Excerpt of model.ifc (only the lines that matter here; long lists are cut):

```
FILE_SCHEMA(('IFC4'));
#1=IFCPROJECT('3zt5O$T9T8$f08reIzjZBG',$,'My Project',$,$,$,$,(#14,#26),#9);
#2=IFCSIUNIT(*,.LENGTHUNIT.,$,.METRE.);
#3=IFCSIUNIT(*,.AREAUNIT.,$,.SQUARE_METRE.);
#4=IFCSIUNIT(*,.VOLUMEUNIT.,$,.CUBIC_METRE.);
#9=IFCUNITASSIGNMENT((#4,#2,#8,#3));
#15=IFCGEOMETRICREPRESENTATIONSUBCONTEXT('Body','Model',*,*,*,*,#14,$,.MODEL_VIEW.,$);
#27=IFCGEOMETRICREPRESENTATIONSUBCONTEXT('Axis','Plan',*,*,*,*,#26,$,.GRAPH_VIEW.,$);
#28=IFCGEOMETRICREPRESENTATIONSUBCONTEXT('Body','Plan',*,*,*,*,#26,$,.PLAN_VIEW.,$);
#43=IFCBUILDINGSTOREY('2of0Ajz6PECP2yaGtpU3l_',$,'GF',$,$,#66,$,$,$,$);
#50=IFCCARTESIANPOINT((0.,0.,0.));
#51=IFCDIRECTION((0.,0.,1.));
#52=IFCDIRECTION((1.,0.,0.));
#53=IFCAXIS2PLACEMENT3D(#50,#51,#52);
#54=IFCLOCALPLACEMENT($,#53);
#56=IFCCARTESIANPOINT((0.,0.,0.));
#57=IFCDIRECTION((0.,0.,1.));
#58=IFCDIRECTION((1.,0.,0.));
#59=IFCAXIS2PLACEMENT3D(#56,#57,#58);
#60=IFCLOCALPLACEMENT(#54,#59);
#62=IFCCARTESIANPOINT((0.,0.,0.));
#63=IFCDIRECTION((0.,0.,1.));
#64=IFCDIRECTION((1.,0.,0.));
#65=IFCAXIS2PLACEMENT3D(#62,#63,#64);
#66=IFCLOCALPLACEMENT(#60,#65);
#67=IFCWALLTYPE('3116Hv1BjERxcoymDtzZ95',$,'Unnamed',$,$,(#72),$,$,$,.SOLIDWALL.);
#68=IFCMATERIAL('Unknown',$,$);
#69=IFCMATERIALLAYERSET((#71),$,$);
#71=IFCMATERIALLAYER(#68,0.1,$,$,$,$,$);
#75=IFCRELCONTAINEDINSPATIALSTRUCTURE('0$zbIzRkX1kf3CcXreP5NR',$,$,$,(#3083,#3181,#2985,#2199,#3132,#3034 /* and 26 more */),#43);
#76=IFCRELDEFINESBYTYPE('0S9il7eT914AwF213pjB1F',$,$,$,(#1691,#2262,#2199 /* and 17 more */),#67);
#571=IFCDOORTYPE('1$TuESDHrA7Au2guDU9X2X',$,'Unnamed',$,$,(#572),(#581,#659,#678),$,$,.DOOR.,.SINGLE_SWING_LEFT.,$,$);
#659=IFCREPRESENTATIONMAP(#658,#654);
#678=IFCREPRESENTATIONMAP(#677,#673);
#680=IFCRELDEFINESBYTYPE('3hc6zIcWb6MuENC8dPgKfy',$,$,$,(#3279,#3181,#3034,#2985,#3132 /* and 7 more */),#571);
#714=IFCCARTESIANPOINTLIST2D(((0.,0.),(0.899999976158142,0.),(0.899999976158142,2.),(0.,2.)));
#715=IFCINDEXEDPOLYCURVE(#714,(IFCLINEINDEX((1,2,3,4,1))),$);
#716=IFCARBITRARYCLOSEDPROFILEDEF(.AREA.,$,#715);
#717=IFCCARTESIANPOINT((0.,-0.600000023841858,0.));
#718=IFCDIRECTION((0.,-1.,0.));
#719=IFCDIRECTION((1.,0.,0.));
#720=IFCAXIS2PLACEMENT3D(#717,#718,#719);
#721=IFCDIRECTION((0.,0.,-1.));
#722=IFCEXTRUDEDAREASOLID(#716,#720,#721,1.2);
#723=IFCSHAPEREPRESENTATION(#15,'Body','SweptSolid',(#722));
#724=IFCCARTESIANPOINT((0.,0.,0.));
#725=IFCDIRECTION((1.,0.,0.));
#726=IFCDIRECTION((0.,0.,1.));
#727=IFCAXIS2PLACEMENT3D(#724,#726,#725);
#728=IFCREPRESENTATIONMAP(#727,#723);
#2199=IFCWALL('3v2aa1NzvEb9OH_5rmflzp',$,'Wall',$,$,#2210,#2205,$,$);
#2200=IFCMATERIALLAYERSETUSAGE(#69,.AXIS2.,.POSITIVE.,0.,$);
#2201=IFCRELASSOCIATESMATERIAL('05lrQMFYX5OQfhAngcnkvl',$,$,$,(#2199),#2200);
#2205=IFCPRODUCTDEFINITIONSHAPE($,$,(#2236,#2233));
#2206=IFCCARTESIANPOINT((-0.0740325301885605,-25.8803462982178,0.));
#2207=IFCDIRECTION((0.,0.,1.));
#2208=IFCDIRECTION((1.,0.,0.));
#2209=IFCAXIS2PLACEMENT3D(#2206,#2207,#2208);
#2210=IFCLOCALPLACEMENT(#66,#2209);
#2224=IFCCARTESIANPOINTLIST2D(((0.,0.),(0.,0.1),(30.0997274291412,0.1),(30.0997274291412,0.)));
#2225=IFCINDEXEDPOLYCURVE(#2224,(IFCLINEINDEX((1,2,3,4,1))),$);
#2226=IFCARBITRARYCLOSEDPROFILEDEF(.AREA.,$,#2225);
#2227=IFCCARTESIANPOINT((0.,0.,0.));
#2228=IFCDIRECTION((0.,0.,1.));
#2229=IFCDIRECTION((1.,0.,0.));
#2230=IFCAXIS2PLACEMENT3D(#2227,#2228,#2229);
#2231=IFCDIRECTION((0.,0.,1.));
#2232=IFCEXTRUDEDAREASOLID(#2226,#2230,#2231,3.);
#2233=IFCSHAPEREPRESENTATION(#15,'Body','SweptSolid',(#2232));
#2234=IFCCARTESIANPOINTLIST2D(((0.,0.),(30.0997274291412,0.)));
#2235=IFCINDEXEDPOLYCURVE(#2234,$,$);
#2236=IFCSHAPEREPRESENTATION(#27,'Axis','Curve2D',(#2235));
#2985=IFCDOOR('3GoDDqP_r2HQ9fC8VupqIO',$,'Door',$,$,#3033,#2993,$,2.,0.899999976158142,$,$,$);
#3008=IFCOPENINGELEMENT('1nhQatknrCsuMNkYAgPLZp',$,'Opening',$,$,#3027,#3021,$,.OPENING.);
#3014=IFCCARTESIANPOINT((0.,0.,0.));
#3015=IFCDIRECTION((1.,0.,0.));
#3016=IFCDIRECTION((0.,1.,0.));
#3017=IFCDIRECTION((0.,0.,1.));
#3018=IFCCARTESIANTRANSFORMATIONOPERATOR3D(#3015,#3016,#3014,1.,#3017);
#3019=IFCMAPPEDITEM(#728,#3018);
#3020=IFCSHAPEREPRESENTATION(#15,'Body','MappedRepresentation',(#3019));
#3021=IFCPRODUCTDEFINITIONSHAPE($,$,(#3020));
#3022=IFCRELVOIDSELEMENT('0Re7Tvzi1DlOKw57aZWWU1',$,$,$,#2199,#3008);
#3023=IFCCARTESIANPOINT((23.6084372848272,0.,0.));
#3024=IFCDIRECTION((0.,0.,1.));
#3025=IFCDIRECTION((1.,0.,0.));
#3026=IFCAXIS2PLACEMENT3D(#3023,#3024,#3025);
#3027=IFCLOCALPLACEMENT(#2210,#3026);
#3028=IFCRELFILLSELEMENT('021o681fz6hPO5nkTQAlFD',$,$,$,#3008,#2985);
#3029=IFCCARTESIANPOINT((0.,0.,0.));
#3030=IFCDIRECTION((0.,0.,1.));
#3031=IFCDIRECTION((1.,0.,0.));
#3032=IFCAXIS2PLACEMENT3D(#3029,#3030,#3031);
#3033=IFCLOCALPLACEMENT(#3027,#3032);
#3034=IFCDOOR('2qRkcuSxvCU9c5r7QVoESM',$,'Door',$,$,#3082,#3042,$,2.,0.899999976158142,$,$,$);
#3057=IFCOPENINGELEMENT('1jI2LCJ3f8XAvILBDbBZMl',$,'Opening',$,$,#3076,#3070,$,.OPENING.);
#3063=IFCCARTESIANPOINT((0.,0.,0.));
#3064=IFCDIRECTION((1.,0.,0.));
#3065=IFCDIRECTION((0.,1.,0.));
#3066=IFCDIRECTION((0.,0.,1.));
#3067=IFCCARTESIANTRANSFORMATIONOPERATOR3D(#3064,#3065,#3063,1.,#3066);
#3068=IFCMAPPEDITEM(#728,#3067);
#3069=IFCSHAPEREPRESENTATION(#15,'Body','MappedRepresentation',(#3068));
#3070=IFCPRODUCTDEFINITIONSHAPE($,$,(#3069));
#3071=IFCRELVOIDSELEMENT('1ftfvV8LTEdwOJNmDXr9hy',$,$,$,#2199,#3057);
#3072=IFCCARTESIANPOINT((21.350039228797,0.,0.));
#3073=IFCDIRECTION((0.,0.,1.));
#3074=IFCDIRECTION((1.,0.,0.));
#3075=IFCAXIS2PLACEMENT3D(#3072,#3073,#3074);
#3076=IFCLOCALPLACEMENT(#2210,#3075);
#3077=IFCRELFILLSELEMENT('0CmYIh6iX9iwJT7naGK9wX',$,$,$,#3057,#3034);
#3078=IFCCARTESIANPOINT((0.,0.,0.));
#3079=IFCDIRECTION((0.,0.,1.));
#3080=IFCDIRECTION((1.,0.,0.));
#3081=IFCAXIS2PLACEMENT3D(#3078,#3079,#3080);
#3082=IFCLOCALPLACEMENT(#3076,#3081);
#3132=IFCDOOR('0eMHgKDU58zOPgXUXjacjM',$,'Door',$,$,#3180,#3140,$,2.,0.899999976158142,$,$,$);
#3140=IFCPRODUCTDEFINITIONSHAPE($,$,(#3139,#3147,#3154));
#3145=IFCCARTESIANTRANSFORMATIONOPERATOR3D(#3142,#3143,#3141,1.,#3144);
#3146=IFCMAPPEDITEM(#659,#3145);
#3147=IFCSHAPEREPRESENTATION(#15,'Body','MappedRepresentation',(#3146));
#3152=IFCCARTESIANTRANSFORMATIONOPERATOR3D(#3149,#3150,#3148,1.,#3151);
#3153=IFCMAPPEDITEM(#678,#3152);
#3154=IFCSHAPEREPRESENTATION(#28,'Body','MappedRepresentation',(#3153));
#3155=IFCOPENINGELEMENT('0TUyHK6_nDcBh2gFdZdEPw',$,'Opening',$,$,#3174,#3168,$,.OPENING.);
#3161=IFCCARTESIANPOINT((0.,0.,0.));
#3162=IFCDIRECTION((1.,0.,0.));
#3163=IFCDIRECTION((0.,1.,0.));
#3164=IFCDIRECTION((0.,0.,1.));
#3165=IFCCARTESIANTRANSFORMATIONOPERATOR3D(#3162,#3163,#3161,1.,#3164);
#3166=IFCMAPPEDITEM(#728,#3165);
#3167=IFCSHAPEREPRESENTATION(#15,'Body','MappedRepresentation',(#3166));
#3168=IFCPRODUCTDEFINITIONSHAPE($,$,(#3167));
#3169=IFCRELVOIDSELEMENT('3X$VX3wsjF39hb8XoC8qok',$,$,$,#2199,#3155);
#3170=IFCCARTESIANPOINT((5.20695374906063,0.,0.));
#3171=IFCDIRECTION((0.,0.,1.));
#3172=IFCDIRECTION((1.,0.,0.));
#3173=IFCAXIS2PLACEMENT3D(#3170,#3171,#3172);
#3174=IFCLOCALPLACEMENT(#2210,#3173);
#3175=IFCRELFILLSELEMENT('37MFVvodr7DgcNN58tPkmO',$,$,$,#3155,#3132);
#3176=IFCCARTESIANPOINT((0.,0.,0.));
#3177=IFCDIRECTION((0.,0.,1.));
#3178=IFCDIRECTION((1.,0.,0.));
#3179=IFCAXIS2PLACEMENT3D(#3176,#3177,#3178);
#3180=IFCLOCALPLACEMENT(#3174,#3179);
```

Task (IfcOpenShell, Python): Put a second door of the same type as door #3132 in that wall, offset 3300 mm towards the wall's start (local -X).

```python
import ifcopenshell
import ifcopenshell.api.feature
import ifcopenshell.api.geometry
import ifcopenshell.api.root
import ifcopenshell.geom
import ifcopenshell.util.element
import ifcopenshell.util.placement
import ifcopenshell.util.shape
import ifcopenshell.util.unit

model = ifcopenshell.open("model.ifc")
unit_scale = ifcopenshell.util.unit.calculate_unit_scale(model)
settings = ifcopenshell.geom.settings()


def volume(element):
    """Net volume in cubic metres, openings subtracted."""
    shape = ifcopenshell.geom.create_shape(settings, element)
    return ifcopenshell.util.shape.get_volume(shape.geometry)


door = model.by_guid("0eMHgKDU58zOPgXUXjacjM")
opening = door.FillsVoids[0].RelatingOpeningElement
wall = opening.VoidsElements[0].RelatingBuildingElement
before = volume(wall)
shift = ifcopenshell.util.placement.get_local_placement(wall.ObjectPlacement)[:3, 0] * -3.3 / unit_scale

# copy_class copies the void relationship, type, container and properties, but no geometry.
new_opening = ifcopenshell.api.root.copy_class(model, product=opening)
new_opening.Representation = ifcopenshell.util.element.copy_deep(
    model, opening.Representation, exclude=["IfcGeometricRepresentationContext", "IfcRepresentationMap"]
)
new_door = ifcopenshell.api.root.copy_class(model, product=door)
new_door.Representation = ifcopenshell.util.element.copy_deep(
    model, door.Representation, exclude=["IfcGeometricRepresentationContext", "IfcRepresentationMap"]
)
ifcopenshell.api.feature.add_filling(model, opening=new_opening, element=new_door)

for old, new in ((opening, new_opening), (door, new_door)):
    matrix = ifcopenshell.util.placement.get_local_placement(old.ObjectPlacement)
    matrix[:3, 3] += shift
    ifcopenshell.api.geometry.edit_object_placement(model, product=new, matrix=matrix, is_si=False)

after = volume(wall)

print(f"wall volume {before:.3f} -> {after:.3f} m3")

model.write("model-out.ifc")
```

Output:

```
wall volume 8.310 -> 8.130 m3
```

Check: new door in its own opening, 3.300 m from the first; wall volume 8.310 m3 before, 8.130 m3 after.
